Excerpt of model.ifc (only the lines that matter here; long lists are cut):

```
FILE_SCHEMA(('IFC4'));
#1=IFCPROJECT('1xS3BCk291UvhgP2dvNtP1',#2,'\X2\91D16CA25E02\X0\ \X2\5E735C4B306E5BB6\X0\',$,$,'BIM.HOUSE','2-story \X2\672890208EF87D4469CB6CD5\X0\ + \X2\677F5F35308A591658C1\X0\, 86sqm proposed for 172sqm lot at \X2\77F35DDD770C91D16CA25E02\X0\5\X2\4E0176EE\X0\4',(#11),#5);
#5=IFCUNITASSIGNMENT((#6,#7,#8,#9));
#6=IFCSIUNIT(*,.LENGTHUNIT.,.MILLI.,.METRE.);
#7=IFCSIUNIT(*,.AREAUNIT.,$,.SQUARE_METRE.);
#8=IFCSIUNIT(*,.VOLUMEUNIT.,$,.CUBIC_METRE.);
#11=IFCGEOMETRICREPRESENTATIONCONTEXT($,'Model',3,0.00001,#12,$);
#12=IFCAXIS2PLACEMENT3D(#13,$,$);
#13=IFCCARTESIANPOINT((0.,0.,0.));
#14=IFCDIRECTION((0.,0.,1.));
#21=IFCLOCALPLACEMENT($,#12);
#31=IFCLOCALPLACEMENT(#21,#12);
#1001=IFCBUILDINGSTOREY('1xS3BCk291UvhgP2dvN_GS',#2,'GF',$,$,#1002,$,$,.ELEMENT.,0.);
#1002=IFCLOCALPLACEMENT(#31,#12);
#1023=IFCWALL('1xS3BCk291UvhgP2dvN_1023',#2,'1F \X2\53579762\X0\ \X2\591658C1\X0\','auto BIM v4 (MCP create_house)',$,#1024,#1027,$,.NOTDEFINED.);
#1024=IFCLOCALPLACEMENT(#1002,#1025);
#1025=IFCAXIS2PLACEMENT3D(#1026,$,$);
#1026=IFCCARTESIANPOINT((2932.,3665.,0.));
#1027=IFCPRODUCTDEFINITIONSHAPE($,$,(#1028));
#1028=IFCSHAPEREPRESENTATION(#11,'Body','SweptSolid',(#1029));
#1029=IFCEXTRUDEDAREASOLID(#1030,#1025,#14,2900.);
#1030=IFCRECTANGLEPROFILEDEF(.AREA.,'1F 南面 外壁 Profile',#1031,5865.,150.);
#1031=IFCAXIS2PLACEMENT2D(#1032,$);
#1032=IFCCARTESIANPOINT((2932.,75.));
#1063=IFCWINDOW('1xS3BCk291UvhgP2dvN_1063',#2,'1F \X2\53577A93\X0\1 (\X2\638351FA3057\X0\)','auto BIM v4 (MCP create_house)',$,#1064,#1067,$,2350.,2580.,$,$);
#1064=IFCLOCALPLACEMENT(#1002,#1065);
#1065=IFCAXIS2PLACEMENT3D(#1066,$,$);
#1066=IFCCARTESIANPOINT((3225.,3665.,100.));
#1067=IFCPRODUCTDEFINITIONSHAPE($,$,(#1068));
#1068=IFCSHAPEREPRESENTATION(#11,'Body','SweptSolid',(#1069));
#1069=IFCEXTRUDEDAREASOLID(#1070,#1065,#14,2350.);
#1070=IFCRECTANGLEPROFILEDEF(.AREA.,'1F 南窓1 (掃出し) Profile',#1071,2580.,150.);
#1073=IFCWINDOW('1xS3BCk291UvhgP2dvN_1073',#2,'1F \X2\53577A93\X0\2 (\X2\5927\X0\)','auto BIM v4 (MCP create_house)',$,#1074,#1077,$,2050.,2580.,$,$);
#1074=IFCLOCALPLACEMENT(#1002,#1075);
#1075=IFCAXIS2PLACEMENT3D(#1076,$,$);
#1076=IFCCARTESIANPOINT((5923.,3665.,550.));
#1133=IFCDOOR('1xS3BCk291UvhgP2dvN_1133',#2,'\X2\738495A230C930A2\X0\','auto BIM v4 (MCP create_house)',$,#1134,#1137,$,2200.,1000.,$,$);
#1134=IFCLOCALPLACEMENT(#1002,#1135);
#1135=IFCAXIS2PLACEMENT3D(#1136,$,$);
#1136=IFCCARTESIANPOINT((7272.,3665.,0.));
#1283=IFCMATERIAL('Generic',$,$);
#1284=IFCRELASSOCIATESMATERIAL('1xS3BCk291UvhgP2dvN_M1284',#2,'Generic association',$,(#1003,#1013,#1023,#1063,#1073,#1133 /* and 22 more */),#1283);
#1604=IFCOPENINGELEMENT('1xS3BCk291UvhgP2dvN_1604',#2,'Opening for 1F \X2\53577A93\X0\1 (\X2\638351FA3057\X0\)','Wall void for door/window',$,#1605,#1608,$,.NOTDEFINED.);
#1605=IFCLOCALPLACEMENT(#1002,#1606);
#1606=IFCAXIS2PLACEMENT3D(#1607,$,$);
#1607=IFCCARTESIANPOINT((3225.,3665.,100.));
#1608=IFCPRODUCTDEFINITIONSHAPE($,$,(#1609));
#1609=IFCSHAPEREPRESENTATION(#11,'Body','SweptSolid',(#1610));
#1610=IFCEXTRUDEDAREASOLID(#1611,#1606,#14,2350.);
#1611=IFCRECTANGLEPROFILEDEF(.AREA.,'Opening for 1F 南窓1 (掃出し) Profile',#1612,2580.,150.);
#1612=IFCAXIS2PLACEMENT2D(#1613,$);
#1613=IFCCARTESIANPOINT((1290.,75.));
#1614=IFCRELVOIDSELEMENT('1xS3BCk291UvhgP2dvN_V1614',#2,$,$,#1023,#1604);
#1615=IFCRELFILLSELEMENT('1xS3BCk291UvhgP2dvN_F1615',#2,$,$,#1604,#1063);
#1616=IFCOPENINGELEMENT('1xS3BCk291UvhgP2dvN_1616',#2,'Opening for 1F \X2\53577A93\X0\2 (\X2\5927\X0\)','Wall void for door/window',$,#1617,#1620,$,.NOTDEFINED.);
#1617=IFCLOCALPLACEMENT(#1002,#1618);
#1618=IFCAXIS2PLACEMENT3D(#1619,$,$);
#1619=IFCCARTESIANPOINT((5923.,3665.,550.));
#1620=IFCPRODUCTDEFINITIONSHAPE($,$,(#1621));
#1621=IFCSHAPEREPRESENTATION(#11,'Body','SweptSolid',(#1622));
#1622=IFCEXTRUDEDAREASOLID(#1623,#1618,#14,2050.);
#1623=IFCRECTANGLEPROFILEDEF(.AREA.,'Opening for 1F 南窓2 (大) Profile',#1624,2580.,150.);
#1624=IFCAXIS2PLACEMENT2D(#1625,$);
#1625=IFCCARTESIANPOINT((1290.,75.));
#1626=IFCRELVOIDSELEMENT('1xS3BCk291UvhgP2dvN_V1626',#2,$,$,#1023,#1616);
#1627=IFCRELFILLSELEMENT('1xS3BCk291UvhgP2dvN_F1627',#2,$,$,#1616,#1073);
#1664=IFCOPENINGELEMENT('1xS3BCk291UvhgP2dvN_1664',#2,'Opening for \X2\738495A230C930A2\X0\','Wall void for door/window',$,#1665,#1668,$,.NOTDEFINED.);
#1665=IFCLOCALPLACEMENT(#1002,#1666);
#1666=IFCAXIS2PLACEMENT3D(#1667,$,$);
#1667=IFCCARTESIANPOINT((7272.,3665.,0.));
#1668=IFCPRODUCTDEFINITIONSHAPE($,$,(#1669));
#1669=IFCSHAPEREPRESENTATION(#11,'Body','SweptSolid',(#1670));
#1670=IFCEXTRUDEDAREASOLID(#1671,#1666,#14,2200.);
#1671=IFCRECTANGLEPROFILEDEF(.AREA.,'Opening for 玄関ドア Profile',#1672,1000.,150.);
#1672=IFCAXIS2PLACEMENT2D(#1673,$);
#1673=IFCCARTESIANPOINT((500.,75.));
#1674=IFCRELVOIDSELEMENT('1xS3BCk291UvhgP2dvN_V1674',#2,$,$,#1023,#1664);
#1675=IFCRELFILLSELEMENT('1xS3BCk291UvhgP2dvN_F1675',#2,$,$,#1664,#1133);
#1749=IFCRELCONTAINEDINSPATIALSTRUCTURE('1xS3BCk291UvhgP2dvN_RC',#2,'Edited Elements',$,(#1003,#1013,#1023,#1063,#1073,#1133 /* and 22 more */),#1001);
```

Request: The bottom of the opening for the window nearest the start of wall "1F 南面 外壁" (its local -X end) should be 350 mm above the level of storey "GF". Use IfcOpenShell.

```python
import numpy as np
import ifcopenshell
import ifcopenshell.api.geometry
import ifcopenshell.geom
import ifcopenshell.util.element
import ifcopenshell.util.placement
import ifcopenshell.util.shape
import ifcopenshell.util.unit

model = ifcopenshell.open("model.ifc")
unit_scale = ifcopenshell.util.unit.calculate_unit_scale(model)

window = model.by_guid("1xS3BCk291UvhgP2dvN_1063")
opening = window.FillsVoids[0].RelatingOpeningElement
storey = ifcopenshell.util.element.get_container(window, ifc_class="IfcBuildingStorey")
level = ifcopenshell.util.placement.get_local_placement(storey.ObjectPlacement)[2, 3]

# The opening's origin need not be at the sill, so measure its lowest point.
shape = ifcopenshell.geom.create_shape(ifcopenshell.geom.settings(), opening)
bottom = ifcopenshell.util.shape.get_shape_bottom_elevation(shape, shape.geometry) / unit_scale
dz = level + 0.35 / unit_scale - bottom

shift = np.array([0.0, 0.0, dz])
# The window is not placed relative to its opening, so move both.
for product in (opening, window):
    matrix = ifcopenshell.util.placement.get_local_placement(product.ObjectPlacement)
    matrix[:3, 3] += shift
    ifcopenshell.api.geometry.edit_object_placement(model, product=product, matrix=matrix, is_si=False)

print(f"moved by {dz * unit_scale:+.3f} m")

model.write("model_edited.ifc")
```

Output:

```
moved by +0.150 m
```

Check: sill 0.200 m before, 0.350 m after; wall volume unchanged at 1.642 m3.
